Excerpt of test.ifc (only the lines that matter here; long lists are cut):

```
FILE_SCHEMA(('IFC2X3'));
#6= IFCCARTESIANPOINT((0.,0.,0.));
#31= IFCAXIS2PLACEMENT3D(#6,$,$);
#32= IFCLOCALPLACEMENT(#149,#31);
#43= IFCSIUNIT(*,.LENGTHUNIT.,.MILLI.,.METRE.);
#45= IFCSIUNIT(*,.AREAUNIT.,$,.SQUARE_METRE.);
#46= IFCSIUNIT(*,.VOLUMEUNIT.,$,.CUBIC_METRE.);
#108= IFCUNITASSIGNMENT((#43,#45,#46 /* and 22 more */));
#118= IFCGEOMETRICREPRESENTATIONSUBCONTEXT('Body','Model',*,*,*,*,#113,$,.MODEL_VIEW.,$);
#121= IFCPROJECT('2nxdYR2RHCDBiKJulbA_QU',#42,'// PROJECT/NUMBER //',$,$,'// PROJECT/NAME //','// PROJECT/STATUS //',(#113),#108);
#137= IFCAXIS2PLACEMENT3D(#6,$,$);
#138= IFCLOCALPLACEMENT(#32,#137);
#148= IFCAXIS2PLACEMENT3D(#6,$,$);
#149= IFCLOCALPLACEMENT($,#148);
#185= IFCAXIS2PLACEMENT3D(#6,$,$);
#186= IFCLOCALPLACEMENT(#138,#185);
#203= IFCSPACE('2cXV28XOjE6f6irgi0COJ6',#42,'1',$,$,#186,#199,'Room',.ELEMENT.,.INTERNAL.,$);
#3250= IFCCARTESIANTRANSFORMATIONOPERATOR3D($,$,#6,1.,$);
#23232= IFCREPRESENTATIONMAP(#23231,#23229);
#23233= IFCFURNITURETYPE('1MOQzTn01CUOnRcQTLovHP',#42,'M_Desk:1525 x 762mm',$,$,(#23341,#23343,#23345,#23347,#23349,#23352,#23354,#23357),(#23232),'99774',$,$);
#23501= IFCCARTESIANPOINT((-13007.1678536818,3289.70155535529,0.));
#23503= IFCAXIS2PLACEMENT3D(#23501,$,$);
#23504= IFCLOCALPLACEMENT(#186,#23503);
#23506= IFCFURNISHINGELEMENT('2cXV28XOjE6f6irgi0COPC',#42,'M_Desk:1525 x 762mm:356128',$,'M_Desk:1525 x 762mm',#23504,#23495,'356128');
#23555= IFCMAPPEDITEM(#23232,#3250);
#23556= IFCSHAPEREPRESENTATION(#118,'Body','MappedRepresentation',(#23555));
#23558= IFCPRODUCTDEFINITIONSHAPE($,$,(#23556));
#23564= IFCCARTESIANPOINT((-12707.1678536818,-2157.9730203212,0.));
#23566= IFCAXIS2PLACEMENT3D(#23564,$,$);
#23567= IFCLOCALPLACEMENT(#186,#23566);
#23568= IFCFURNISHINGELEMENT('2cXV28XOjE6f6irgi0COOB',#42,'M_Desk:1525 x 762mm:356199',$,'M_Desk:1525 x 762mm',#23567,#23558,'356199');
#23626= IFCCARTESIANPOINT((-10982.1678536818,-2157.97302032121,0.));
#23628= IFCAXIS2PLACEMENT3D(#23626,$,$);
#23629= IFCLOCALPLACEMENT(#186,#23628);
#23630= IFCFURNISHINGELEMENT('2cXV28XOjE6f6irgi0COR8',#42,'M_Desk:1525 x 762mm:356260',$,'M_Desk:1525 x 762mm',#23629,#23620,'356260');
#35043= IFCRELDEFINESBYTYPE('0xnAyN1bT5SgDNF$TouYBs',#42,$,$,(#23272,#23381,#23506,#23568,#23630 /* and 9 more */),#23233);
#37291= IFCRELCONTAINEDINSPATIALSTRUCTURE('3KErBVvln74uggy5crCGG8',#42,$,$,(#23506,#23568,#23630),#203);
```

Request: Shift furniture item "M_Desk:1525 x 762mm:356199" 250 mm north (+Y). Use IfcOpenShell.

```python
import ifcopenshell
import ifcopenshell.api.geometry
import ifcopenshell.util.placement

model = ifcopenshell.open("test.ifc")

item = model.by_guid("2cXV28XOjE6f6irgi0COOB")
matrix = ifcopenshell.util.placement.get_local_placement(item.ObjectPlacement)
matrix[1, 3] += 250.0
ifcopenshell.api.geometry.edit_object_placement(model, product=item, matrix=matrix, is_si=False)

print(ifcopenshell.util.placement.get_local_placement(item.ObjectPlacement).round(3) + 0.0)

model.write("test_updated.ifc")
```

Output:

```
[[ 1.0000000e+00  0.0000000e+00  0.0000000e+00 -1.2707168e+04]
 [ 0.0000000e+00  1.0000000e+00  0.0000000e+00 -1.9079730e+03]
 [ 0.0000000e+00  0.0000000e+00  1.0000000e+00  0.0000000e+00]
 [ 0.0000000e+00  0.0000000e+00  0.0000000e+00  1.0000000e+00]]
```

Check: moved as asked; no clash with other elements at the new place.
